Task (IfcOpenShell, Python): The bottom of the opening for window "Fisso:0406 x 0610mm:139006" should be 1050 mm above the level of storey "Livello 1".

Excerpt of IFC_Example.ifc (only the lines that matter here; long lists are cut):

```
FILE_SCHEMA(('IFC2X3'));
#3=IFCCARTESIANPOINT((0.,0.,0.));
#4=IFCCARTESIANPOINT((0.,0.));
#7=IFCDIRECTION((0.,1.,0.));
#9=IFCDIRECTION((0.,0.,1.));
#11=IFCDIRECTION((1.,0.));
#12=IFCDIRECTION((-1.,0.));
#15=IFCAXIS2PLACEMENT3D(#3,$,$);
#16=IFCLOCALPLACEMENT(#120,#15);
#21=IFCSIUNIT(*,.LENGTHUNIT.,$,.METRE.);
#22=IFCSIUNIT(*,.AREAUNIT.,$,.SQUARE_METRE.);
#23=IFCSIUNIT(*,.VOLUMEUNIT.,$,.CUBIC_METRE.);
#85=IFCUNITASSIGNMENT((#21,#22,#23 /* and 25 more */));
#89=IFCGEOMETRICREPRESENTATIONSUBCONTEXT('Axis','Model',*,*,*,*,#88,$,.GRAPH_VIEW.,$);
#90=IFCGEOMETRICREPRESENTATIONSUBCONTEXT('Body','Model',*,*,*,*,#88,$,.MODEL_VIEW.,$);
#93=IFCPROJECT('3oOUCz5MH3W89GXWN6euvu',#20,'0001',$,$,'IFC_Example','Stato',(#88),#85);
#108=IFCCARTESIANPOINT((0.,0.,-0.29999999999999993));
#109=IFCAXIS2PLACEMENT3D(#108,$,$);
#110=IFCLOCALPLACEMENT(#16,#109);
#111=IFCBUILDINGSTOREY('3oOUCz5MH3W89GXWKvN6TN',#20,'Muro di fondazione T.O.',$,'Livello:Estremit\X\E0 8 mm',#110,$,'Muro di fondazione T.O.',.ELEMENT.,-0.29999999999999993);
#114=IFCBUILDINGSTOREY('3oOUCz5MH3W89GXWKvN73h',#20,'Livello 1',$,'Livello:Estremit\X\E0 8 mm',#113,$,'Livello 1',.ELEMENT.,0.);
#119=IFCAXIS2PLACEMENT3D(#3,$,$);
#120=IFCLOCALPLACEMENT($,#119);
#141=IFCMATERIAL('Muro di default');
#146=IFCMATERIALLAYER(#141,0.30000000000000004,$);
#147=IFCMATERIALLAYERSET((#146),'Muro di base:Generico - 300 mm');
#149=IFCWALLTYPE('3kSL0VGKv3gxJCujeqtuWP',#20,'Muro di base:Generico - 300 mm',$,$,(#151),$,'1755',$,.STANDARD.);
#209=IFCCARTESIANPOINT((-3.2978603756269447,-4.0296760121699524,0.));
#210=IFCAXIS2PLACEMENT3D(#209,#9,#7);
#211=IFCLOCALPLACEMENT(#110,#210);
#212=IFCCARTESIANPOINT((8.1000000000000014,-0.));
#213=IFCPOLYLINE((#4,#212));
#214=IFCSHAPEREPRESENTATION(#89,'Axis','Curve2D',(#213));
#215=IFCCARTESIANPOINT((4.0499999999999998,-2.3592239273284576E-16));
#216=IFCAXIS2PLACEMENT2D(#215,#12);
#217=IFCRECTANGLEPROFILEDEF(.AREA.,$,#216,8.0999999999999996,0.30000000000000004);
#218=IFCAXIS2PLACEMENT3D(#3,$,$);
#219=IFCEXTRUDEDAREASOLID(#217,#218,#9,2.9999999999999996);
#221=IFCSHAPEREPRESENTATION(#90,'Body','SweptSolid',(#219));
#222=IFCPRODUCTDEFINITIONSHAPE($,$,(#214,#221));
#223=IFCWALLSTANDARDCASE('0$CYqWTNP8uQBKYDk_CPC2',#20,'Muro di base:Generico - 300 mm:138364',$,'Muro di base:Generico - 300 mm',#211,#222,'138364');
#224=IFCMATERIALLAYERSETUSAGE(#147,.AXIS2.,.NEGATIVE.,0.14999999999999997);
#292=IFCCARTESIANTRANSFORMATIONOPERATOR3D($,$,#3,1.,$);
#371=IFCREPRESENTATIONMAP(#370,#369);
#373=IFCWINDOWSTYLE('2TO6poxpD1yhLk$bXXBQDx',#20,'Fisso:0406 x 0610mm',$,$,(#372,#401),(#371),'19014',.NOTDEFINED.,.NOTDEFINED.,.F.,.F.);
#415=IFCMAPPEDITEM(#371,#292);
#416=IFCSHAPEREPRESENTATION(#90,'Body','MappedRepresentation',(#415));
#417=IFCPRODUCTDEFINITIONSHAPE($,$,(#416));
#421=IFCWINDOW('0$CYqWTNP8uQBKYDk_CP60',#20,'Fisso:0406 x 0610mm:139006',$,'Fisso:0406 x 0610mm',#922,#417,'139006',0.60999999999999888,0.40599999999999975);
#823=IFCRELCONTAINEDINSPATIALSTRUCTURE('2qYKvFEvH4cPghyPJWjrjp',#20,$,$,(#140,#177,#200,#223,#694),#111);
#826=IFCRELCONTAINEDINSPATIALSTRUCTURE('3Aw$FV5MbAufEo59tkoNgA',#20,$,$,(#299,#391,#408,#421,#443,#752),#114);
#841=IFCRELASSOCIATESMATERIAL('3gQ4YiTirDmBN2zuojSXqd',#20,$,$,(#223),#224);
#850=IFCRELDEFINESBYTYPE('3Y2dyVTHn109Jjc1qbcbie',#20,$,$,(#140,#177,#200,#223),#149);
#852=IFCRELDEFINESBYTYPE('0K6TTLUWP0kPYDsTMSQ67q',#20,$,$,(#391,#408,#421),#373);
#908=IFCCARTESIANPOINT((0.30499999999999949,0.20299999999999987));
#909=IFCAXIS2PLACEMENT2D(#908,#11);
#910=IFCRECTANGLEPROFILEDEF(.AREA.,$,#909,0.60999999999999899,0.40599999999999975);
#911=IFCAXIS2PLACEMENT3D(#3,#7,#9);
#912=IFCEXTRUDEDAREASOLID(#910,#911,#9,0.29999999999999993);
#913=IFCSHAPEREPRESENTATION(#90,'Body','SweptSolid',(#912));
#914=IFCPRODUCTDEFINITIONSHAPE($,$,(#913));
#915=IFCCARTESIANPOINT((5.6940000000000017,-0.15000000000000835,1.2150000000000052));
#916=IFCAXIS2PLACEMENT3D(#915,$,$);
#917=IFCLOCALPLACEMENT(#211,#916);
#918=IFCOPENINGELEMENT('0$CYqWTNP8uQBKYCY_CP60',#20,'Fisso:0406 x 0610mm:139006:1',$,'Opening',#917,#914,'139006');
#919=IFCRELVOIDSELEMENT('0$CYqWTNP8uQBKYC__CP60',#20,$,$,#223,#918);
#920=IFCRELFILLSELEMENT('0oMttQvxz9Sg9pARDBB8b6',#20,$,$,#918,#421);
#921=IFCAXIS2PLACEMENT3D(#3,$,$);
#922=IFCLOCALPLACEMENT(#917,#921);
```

```python
import numpy as np
import ifcopenshell
import ifcopenshell.api.geometry
import ifcopenshell.geom
import ifcopenshell.util.element
import ifcopenshell.util.placement
import ifcopenshell.util.shape
import ifcopenshell.util.unit

model = ifcopenshell.open("IFC_Example.ifc")
unit_scale = ifcopenshell.util.unit.calculate_unit_scale(model)

window = model.by_id(421)
opening = window.FillsVoids[0].RelatingOpeningElement
storey = ifcopenshell.util.element.get_container(window, ifc_class="IfcBuildingStorey")
level = ifcopenshell.util.placement.get_local_placement(storey.ObjectPlacement)[2, 3]

# The opening's origin need not be at the sill, so measure its lowest point.
shape = ifcopenshell.geom.create_shape(ifcopenshell.geom.settings(), opening)
bottom = ifcopenshell.util.shape.get_shape_bottom_elevation(shape, shape.geometry) / unit_scale
dz = level + 1.05 / unit_scale - bottom

shift = np.array([0.0, 0.0, dz])
# The window is placed relative to its opening, so it follows when the opening moves.
matrix = ifcopenshell.util.placement.get_local_placement(opening.ObjectPlacement)
matrix[:3, 3] += shift
ifcopenshell.api.geometry.edit_object_placement(
    model, product=opening, matrix=matrix, is_si=False, should_transform_children=True
)

print(f"moved by {dz * unit_scale:+.3f} m")

model.write("IFC_Example_v2.ifc")
```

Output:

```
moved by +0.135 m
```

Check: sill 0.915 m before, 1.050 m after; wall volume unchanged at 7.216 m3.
